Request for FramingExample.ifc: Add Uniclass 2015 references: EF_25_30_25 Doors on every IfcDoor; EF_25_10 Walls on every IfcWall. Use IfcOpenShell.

First a look at what the model holds.

```python
import ifcopenshell

model = ifcopenshell.open("FramingExample.ifc")
print(model.schema)
print("classifications:", [c.Name for c in model.by_type("IfcClassification")])
for ifc_class in ("IfcDoor", "IfcRoof", "IfcStair", "IfcWall", "IfcWindow"):
    print(ifc_class, len(model.by_type(ifc_class)))
```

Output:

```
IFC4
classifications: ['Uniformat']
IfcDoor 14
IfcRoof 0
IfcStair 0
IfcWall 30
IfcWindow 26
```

```python
import ifcopenshell
import ifcopenshell.api.classification

model = ifcopenshell.open("FramingExample.ifc")

system = ifcopenshell.api.classification.add_classification(model, classification="Uniclass 2015")

codes = {
    "IfcDoor": ("EF_25_30_25", "Doors"),
    "IfcWall": ("EF_25_10", "Walls"),
}
for ifc_class, (code, name) in codes.items():
    products = model.by_type(ifc_class)
    ifcopenshell.api.classification.add_reference(
        model, products=products, classification=system, identification=code, name=name
    )
    print(code, len(products))

model.write("FramingExample-out.ifc")
```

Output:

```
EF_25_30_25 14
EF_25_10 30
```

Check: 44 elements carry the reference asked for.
